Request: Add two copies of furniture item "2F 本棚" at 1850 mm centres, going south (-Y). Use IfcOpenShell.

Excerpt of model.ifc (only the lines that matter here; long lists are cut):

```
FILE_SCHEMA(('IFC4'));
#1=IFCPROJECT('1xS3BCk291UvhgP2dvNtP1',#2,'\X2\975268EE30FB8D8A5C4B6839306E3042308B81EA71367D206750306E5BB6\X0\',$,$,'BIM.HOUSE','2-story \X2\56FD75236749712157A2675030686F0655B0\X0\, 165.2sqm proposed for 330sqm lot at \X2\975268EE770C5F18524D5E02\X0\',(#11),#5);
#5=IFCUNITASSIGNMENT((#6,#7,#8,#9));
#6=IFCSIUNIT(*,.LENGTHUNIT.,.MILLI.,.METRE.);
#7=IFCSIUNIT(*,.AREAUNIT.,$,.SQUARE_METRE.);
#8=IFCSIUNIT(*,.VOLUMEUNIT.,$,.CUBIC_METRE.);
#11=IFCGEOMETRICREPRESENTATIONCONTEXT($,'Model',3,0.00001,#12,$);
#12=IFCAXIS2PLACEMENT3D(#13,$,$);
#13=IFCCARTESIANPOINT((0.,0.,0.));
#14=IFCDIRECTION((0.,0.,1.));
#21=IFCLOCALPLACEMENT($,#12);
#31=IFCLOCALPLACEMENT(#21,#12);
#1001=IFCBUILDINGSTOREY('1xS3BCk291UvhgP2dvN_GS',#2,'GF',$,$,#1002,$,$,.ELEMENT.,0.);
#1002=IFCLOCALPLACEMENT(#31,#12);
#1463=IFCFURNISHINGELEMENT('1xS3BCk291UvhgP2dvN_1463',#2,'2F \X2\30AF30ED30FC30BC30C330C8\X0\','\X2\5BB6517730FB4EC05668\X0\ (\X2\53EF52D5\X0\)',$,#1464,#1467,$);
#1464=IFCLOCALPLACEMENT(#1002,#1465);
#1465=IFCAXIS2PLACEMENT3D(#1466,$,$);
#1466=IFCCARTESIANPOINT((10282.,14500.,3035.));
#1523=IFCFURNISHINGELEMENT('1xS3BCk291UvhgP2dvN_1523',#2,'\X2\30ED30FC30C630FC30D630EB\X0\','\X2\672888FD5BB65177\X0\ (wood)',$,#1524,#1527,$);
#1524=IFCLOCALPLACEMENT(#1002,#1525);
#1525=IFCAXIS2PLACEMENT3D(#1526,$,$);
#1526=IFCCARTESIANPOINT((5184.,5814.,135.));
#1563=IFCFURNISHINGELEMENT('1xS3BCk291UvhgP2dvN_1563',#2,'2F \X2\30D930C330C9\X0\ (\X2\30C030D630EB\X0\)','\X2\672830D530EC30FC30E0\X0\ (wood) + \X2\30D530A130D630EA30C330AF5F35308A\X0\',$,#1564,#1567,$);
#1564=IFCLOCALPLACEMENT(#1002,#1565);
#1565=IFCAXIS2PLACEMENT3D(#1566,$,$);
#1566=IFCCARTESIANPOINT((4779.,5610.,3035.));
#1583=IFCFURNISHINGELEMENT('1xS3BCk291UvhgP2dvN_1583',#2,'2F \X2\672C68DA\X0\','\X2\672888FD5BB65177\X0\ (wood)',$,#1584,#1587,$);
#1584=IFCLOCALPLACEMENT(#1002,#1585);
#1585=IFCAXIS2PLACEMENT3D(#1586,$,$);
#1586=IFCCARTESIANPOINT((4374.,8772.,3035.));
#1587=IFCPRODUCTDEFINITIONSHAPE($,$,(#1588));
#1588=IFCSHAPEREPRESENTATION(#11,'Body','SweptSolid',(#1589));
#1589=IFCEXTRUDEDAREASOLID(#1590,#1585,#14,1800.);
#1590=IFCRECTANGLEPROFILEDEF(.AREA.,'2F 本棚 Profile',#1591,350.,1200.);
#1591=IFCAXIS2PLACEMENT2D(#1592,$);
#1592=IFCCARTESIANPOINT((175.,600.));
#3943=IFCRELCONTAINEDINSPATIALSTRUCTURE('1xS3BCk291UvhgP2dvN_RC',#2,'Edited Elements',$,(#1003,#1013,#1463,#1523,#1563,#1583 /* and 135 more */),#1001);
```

```python
import numpy as np
import ifcopenshell
import ifcopenshell.api.geometry
import ifcopenshell.api.root
import ifcopenshell.util.element
import ifcopenshell.util.placement

model = ifcopenshell.open("model.ifc")


def reuse_history(source, copy):
    """copy_class also copies each property set's owner history, people and application; keep the originals."""
    for rel in copy.IsDefinedBy:
        if rel.is_a("IfcRelDefinesByProperties") and (history := rel.RelatingPropertyDefinition.OwnerHistory):
            rel.RelatingPropertyDefinition.OwnerHistory = source.OwnerHistory
            ifcopenshell.util.element.remove_deep2(model, history)


source = model.by_id(1583)
base = ifcopenshell.util.placement.get_local_placement(source.ObjectPlacement)
step = np.array([0.0, -1.0, 0.0]) * 1850.0

for i in range(1, 3):
    copy = ifcopenshell.api.root.copy_class(model, product=source)
    copy.Representation = ifcopenshell.util.element.copy_deep(
        model, source.Representation, exclude=["IfcGeometricRepresentationContext", "IfcRepresentationMap"]
    )
    reuse_history(source, copy)
    matrix = base.copy()
    matrix[:3, 3] += i * step
    print("added at", matrix[:3, 3].round(3) + 0.0)
    ifcopenshell.api.geometry.edit_object_placement(model, product=copy, matrix=matrix, is_si=False)

model.write("model_edited.ifc")
```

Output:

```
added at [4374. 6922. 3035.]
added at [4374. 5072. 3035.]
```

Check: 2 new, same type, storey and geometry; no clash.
